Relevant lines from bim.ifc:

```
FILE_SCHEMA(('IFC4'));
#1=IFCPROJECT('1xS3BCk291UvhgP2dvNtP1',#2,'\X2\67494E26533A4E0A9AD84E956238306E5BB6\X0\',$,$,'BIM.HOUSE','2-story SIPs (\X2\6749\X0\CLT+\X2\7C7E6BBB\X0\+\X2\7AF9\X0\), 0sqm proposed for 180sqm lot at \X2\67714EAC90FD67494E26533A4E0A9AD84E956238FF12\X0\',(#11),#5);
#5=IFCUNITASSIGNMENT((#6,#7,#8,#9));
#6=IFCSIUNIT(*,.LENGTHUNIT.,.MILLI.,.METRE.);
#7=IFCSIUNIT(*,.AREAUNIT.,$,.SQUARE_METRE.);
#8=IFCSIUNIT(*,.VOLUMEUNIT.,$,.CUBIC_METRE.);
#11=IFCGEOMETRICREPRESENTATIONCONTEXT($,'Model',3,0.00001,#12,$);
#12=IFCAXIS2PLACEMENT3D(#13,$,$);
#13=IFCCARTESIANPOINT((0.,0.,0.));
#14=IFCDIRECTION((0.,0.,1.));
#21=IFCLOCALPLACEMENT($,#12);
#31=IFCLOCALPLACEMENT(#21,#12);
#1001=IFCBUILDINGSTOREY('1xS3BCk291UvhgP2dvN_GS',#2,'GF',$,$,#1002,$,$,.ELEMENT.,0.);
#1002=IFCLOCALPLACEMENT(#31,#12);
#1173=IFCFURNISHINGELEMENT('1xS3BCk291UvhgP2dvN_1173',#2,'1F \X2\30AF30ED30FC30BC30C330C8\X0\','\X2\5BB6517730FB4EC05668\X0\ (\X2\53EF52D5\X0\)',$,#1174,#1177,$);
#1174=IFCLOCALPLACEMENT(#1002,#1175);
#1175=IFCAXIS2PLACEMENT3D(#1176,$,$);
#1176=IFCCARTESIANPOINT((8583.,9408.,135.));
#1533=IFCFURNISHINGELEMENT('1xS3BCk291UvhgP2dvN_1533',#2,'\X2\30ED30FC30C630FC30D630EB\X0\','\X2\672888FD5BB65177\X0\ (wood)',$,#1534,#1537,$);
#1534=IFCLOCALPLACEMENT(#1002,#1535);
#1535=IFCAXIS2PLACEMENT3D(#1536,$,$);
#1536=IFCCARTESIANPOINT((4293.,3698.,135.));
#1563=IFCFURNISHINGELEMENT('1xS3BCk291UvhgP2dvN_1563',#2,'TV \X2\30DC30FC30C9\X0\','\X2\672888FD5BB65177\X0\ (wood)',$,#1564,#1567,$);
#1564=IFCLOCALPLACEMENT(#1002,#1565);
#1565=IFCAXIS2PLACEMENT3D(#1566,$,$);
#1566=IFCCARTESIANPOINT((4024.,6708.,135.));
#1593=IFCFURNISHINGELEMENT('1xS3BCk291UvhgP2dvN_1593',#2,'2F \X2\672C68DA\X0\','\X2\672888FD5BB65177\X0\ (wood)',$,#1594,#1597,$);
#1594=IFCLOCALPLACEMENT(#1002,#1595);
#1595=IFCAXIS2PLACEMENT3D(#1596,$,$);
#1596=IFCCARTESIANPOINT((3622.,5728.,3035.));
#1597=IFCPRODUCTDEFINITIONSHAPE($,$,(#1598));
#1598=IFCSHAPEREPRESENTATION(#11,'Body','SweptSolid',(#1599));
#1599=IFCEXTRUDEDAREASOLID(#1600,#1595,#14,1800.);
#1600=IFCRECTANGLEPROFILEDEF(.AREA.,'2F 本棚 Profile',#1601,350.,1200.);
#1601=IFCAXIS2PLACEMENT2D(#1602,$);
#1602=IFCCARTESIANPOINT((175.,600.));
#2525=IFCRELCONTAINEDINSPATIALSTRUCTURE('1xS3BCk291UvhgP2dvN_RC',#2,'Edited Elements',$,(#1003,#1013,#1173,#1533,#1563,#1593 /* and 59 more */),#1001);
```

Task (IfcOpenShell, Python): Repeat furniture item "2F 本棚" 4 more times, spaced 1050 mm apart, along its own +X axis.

```python
import ifcopenshell
import ifcopenshell.api.geometry
import ifcopenshell.api.root
import ifcopenshell.util.element
import ifcopenshell.util.placement

model = ifcopenshell.open("bim.ifc")


def reuse_history(source, copy):
    """copy_class also copies each property set's owner history, people and application; keep the originals."""
    for rel in copy.IsDefinedBy:
        if rel.is_a("IfcRelDefinesByProperties") and (history := rel.RelatingPropertyDefinition.OwnerHistory):
            rel.RelatingPropertyDefinition.OwnerHistory = source.OwnerHistory
            ifcopenshell.util.element.remove_deep2(model, history)


source = model.by_id(1593)
base = ifcopenshell.util.placement.get_local_placement(source.ObjectPlacement)
step = base[:3, 0] * 1050.0

for i in range(1, 5):
    copy = ifcopenshell.api.root.copy_class(model, product=source)
    copy.Representation = ifcopenshell.util.element.copy_deep(
        model, source.Representation, exclude=["IfcGeometricRepresentationContext", "IfcRepresentationMap"]
    )
    reuse_history(source, copy)
    matrix = base.copy()
    matrix[:3, 3] += i * step
    print("added at", matrix[:3, 3].round(3) + 0.0)
    ifcopenshell.api.geometry.edit_object_placement(model, product=copy, matrix=matrix, is_si=False)

model.write("bim_v2.ifc")
```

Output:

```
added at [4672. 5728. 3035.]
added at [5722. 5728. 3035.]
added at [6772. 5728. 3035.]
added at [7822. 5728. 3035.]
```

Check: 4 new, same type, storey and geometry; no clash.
